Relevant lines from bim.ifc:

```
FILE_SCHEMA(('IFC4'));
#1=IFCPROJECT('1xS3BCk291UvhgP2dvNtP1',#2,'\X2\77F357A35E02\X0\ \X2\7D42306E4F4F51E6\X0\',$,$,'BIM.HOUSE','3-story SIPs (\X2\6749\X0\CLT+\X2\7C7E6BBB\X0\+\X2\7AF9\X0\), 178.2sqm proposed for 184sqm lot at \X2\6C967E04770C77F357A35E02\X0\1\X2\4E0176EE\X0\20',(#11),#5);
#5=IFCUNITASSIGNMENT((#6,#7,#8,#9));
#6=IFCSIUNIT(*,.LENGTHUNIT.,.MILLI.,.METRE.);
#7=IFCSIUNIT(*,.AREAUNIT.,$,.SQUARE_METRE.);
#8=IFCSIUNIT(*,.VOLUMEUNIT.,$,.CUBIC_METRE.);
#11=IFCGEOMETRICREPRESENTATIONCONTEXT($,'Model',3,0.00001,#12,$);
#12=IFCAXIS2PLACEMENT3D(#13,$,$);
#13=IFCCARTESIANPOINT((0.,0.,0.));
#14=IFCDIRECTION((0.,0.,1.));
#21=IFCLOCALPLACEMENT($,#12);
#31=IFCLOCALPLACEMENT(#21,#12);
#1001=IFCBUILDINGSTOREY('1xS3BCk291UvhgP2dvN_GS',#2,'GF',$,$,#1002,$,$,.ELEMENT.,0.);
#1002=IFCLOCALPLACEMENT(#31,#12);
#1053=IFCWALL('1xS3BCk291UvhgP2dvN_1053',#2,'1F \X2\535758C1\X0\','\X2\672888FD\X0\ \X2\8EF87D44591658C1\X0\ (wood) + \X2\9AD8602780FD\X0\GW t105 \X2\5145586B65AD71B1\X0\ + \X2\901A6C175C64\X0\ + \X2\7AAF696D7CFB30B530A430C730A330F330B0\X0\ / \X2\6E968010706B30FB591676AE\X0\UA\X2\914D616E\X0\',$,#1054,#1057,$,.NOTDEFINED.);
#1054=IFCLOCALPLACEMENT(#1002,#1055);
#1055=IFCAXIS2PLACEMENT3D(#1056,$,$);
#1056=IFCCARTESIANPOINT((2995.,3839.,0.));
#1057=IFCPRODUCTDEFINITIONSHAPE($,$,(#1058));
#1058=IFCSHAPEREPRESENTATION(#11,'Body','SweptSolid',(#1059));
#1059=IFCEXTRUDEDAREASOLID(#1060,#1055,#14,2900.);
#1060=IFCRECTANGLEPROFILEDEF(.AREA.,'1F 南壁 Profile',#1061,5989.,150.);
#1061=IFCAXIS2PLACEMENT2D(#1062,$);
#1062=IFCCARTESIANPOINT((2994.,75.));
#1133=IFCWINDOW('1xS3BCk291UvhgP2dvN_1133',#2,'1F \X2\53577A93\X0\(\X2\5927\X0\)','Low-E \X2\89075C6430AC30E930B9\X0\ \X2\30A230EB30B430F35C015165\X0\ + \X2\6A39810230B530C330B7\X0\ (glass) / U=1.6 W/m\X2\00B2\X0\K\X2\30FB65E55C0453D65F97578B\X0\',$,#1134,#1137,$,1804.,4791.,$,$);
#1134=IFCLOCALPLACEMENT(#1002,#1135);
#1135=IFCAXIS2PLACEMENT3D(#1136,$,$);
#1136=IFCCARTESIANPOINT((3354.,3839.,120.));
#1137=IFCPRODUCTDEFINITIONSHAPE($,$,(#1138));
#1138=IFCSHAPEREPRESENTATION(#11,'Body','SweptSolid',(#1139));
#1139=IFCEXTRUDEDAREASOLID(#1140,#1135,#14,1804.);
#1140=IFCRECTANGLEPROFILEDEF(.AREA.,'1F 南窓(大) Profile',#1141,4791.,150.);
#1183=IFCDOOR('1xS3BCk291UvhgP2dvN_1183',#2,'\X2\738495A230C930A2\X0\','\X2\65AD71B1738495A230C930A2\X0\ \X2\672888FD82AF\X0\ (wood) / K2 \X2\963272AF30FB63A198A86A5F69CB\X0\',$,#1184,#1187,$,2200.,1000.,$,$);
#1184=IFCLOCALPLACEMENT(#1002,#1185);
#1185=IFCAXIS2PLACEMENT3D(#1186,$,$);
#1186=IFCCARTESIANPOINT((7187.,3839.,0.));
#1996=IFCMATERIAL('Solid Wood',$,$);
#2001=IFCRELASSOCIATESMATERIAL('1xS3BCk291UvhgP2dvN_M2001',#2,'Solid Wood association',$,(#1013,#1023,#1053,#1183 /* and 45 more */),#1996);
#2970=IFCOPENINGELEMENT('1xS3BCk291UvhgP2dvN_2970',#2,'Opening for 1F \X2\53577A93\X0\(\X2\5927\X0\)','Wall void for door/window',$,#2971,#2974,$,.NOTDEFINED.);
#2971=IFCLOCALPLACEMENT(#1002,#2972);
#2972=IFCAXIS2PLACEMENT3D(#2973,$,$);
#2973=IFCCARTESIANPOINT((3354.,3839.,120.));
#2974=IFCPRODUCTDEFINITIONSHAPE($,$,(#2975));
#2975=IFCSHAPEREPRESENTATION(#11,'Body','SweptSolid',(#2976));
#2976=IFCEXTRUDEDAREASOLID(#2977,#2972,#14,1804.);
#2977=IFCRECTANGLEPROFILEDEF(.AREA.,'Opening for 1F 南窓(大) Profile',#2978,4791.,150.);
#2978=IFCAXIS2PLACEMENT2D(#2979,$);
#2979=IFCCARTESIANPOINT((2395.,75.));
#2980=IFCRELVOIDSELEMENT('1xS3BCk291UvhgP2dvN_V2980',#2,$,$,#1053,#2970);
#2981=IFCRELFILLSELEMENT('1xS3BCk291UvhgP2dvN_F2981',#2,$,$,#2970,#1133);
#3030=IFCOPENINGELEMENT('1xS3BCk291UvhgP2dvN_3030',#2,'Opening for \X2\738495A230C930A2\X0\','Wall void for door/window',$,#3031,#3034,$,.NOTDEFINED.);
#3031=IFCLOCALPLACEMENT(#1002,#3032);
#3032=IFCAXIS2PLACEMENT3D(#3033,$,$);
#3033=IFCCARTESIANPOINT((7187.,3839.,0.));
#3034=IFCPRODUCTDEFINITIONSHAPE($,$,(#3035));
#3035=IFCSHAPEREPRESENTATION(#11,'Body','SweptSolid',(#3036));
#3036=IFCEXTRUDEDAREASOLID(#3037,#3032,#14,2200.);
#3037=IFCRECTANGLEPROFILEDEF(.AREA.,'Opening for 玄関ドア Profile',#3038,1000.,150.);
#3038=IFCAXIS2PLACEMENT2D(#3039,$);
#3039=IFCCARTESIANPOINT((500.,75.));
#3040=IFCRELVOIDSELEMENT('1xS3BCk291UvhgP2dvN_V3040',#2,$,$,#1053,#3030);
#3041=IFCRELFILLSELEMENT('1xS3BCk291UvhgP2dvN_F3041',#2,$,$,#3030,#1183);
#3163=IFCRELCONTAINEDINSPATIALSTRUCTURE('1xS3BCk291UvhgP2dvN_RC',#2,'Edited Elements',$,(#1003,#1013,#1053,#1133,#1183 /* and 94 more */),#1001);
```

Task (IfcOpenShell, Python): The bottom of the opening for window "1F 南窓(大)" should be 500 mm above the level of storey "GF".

```python
import numpy as np
import ifcopenshell
import ifcopenshell.api.geometry
import ifcopenshell.geom
import ifcopenshell.util.element
import ifcopenshell.util.placement
import ifcopenshell.util.shape
import ifcopenshell.util.unit

model = ifcopenshell.open("bim.ifc")
unit_scale = ifcopenshell.util.unit.calculate_unit_scale(model)

window = model.by_guid("1xS3BCk291UvhgP2dvN_1133")
opening = window.FillsVoids[0].RelatingOpeningElement
storey = ifcopenshell.util.element.get_container(window, ifc_class="IfcBuildingStorey")
level = ifcopenshell.util.placement.get_local_placement(storey.ObjectPlacement)[2, 3]

# The opening's origin need not be at the sill, so measure its lowest point.
shape = ifcopenshell.geom.create_shape(ifcopenshell.geom.settings(), opening)
bottom = ifcopenshell.util.shape.get_shape_bottom_elevation(shape, shape.geometry) / unit_scale
dz = level + 0.5 / unit_scale - bottom

shift = np.array([0.0, 0.0, dz])
# The window is not placed relative to its opening, so move both.
for product in (opening, window):
    matrix = ifcopenshell.util.placement.get_local_placement(product.ObjectPlacement)
    matrix[:3, 3] += shift
    ifcopenshell.api.geometry.edit_object_placement(model, product=product, matrix=matrix, is_si=False)

print(f"moved by {dz * unit_scale:+.3f} m")

model.write("bim_updated.ifc")
```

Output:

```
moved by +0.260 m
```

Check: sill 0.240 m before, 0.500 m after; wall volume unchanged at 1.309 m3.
